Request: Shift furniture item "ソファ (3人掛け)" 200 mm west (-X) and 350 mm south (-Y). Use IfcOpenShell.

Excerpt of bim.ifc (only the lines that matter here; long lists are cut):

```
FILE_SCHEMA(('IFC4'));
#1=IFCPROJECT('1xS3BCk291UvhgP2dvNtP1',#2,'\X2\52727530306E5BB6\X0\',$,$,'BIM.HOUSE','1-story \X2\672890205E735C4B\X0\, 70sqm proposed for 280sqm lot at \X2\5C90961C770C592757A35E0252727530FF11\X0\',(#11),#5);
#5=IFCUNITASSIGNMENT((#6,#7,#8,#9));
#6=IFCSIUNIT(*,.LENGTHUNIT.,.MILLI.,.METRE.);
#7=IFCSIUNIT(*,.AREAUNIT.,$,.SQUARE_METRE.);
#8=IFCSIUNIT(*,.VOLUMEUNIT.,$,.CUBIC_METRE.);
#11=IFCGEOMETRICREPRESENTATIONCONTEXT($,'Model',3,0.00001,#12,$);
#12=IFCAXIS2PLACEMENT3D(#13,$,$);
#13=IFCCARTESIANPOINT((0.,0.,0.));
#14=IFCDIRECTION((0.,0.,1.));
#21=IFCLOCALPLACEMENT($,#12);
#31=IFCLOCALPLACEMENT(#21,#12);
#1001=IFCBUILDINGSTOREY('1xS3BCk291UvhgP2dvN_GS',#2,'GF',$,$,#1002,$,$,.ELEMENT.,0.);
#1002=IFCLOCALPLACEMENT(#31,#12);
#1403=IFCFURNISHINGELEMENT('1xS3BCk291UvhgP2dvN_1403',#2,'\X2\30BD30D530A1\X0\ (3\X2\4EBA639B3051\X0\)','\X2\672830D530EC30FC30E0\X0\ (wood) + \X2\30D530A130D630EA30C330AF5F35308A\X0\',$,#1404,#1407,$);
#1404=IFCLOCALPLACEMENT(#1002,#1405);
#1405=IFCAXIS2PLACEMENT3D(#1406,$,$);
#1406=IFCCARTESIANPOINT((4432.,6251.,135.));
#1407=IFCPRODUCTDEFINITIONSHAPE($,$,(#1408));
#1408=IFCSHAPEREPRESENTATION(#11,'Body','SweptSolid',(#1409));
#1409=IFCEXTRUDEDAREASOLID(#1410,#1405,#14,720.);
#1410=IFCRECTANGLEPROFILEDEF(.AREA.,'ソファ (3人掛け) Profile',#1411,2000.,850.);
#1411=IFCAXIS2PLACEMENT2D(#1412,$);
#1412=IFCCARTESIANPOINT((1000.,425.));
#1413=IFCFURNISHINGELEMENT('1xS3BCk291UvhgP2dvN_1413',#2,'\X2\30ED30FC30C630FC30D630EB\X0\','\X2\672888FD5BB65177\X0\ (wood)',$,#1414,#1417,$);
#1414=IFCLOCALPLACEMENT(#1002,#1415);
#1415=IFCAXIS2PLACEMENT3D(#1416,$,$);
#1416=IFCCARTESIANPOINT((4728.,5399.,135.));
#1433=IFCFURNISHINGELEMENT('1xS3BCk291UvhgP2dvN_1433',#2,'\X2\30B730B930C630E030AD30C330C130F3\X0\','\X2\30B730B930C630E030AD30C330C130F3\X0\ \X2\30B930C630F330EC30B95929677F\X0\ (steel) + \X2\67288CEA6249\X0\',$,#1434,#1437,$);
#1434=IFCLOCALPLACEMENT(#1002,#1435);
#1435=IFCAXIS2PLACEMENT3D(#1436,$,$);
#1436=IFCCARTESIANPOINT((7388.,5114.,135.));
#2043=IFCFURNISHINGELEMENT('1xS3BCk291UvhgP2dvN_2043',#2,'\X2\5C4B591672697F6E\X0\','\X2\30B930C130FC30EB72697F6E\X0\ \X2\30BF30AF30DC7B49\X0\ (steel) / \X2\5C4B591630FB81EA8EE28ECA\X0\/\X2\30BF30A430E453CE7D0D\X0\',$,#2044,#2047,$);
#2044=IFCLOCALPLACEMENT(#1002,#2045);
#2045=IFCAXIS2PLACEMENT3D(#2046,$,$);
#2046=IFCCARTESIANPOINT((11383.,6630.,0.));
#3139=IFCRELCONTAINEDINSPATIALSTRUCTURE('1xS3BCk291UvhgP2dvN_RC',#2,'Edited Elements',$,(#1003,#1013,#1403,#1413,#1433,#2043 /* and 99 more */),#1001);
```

```python
import ifcopenshell
import ifcopenshell.api.geometry
import ifcopenshell.util.placement
import ifcopenshell.util.unit

model = ifcopenshell.open("bim.ifc")
unit_scale = ifcopenshell.util.unit.calculate_unit_scale(model)

item = model.by_guid("1xS3BCk291UvhgP2dvN_1403")
matrix = ifcopenshell.util.placement.get_local_placement(item.ObjectPlacement)
matrix[0, 3] -= 0.2 / unit_scale
matrix[1, 3] -= 0.35 / unit_scale
ifcopenshell.api.geometry.edit_object_placement(model, product=item, matrix=matrix, is_si=False)

print(ifcopenshell.util.placement.get_local_placement(item.ObjectPlacement).round(3) + 0.0)

model.write("bim_v2.ifc")
```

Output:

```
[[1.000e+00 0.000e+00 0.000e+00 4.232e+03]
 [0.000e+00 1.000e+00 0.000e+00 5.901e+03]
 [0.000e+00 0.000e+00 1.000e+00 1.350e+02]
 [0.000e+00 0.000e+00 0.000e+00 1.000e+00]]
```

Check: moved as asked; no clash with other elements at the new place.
